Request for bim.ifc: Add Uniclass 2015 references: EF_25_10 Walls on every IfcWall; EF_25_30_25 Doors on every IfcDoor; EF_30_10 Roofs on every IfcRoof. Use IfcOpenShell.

First a look at what the model holds.

```python
import ifcopenshell

model = ifcopenshell.open("bim.ifc")
print(model.schema)
print("classifications:", [c.Name for c in model.by_type("IfcClassification")])
for ifc_class in ("IfcDoor", "IfcRoof", "IfcStair", "IfcWall", "IfcWindow"):
    print(ifc_class, len(model.by_type(ifc_class)))
```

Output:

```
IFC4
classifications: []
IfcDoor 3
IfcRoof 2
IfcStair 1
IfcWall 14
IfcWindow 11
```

```python
import ifcopenshell
import ifcopenshell.api.classification

model = ifcopenshell.open("bim.ifc")

system = ifcopenshell.api.classification.add_classification(model, classification="Uniclass 2015")

codes = {
    "IfcWall": ("EF_25_10", "Walls"),
    "IfcDoor": ("EF_25_30_25", "Doors"),
    "IfcRoof": ("EF_30_10", "Roofs"),
}
for ifc_class, (code, name) in codes.items():
    products = model.by_type(ifc_class)
    ifcopenshell.api.classification.add_reference(
        model, products=products, classification=system, identification=code, name=name
    )
    print(code, len(products))

model.write("bim-out.ifc")
```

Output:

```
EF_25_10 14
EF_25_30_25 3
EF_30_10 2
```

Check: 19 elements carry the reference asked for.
